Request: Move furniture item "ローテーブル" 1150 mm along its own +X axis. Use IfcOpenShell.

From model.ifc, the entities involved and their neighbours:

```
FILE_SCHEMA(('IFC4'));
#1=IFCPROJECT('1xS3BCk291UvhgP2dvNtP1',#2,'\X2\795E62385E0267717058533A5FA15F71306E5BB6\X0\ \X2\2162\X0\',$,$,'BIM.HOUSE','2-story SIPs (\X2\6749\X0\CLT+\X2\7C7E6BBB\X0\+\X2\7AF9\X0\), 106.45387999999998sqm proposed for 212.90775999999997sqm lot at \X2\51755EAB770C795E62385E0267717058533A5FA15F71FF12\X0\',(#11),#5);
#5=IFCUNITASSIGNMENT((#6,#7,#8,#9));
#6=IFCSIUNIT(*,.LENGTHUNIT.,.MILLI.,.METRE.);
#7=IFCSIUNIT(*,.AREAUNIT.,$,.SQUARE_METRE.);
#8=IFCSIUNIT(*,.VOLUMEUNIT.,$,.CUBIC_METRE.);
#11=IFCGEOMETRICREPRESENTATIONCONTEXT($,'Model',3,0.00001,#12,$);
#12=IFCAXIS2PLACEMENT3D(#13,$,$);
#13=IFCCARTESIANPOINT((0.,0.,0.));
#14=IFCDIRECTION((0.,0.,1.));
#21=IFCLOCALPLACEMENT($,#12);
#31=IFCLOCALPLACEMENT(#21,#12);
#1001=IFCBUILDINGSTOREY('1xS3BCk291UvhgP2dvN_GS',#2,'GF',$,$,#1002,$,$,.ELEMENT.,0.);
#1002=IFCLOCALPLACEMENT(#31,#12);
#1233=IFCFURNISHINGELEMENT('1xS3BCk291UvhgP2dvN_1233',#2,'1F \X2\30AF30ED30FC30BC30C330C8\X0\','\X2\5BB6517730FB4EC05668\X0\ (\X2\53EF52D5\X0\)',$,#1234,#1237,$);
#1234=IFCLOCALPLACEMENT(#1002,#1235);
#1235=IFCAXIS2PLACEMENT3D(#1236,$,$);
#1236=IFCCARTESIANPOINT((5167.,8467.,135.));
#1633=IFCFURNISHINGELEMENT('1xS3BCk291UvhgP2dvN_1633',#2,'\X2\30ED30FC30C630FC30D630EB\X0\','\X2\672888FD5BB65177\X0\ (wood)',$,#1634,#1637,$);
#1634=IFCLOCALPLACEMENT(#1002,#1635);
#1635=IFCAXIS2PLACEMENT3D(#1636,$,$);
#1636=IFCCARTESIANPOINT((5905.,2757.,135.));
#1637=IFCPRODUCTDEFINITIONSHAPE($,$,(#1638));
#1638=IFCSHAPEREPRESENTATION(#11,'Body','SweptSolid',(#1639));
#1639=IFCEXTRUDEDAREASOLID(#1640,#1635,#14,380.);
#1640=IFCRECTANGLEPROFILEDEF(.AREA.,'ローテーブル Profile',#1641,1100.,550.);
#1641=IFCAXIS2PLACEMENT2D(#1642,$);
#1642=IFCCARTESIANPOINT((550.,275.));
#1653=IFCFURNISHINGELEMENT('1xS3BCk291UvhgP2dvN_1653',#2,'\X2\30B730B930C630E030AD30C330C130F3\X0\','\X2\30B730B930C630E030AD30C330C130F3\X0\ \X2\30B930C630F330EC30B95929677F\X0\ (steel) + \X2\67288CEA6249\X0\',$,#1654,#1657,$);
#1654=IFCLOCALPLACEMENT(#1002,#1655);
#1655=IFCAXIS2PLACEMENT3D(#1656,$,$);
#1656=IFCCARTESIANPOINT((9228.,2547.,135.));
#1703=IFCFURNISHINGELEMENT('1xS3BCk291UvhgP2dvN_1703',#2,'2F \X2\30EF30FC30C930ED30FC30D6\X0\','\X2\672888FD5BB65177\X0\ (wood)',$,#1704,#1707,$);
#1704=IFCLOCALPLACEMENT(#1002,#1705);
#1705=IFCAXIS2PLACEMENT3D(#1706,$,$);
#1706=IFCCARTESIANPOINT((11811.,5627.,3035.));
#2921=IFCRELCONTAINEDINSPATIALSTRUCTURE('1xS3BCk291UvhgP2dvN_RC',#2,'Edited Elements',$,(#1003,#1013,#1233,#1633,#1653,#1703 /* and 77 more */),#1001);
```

```python
import ifcopenshell
import ifcopenshell.api.geometry
import ifcopenshell.util.placement

model = ifcopenshell.open("model.ifc")

item = model.by_id(1633)
matrix = ifcopenshell.util.placement.get_local_placement(item.ObjectPlacement)
matrix[:3, 3] += matrix[:3, 0] * 1150.0
ifcopenshell.api.geometry.edit_object_placement(model, product=item, matrix=matrix, is_si=False)

print(ifcopenshell.util.placement.get_local_placement(item.ObjectPlacement).round(3) + 0.0)

model.write("model_rev.ifc")
```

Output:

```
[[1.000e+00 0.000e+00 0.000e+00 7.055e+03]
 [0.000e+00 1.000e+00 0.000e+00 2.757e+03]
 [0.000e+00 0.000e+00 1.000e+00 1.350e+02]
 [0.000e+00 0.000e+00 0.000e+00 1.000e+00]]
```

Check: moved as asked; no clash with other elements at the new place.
